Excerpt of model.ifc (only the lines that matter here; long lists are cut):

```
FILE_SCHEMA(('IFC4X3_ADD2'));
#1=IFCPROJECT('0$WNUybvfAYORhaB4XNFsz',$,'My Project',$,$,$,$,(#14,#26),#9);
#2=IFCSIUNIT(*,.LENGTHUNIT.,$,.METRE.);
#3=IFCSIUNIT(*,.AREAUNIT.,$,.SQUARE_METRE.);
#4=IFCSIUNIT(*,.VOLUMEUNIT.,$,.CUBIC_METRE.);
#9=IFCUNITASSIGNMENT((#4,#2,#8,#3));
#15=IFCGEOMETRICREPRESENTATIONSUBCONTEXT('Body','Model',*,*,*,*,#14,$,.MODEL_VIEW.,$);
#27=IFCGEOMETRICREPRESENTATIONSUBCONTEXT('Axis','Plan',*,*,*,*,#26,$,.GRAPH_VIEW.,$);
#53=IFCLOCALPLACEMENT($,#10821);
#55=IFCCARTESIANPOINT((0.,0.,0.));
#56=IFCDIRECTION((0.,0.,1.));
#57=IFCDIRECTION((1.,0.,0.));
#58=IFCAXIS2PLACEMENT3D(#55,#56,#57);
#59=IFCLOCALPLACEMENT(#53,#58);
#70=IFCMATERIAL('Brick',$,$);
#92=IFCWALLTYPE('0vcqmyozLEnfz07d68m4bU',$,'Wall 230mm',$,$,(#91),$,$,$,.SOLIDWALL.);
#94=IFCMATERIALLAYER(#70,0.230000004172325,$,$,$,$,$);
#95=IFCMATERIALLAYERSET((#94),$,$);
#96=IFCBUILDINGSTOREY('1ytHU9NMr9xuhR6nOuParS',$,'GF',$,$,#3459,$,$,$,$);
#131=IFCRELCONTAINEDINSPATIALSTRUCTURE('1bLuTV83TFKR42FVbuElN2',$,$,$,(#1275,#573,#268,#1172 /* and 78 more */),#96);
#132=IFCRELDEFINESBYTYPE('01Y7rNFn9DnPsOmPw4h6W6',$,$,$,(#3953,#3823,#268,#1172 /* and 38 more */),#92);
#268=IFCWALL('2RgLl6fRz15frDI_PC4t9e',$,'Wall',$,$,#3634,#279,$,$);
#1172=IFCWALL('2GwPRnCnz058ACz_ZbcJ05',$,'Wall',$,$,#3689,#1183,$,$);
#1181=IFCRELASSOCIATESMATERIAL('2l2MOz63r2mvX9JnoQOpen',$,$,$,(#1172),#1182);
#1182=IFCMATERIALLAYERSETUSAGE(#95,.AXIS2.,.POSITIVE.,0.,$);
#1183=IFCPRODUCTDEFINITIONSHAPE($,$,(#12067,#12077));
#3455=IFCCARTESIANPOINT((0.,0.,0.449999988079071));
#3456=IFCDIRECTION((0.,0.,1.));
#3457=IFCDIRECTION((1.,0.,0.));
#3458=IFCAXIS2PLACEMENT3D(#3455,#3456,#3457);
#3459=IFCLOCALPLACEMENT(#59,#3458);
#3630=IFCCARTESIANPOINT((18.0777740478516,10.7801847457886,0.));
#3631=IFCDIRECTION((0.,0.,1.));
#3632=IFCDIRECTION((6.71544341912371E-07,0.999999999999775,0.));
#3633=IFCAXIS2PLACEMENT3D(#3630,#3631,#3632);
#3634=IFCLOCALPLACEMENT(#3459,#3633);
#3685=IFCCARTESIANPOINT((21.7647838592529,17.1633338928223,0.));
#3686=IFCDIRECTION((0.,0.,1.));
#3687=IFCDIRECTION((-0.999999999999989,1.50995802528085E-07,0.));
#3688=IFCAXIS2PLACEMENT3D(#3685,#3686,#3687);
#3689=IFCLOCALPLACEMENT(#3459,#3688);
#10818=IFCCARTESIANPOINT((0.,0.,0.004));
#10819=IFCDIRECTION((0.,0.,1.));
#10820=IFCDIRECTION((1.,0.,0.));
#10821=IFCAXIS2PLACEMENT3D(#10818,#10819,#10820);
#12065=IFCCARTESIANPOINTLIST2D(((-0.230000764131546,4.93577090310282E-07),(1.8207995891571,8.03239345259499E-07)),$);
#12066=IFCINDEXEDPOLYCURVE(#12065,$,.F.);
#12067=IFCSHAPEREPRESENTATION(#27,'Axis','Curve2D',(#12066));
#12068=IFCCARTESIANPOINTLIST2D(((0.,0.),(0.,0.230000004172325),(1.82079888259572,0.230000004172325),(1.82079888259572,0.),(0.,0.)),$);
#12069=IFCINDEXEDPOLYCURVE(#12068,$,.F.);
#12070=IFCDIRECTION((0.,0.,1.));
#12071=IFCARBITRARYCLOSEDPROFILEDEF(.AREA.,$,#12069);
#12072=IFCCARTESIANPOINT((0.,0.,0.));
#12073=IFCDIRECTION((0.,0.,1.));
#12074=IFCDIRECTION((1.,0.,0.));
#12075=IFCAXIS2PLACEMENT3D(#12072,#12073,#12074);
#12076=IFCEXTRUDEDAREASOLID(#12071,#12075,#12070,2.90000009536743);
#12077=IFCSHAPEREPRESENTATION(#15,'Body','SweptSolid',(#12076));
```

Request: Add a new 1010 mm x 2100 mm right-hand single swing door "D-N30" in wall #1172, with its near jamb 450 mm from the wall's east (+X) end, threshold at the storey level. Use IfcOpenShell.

```python
import numpy as np
import ifcopenshell
import ifcopenshell.api.feature
import ifcopenshell.api.geometry
import ifcopenshell.api.root
import ifcopenshell.api.spatial
import ifcopenshell.geom
import ifcopenshell.util.element
import ifcopenshell.util.placement
import ifcopenshell.util.representation
import ifcopenshell.util.shape
import ifcopenshell.util.unit

model = ifcopenshell.open("model.ifc")
unit_scale = ifcopenshell.util.unit.calculate_unit_scale(model)
settings = ifcopenshell.geom.settings()


def volume(element):
    """Net volume in cubic metres, openings subtracted."""
    shape = ifcopenshell.geom.create_shape(settings, element)
    return ifcopenshell.util.shape.get_volume(shape.geometry)


wall = model.by_id(1172)
storey = ifcopenshell.util.element.get_container(wall, ifc_class="IfcBuildingStorey")
context = ifcopenshell.util.representation.get_context(model, "Model", "Body", "MODEL_VIEW")
before = volume(wall)

width, height, from_end, sill = 1.01, 2.1, 0.45, 0.0  # metres

# The wall runs along its own X axis, and the end named is its -X end.
wall_shape = ifcopenshell.geom.create_shape(settings, wall)
x, y, z = ifcopenshell.util.shape.get_vertices(wall_shape.geometry).T
start = x.min() + from_end
face, thickness = float(y.min()), float(y.max() - y.min())
wall_matrix = ifcopenshell.util.placement.get_local_placement(wall.ObjectPlacement)
level = ifcopenshell.util.placement.get_local_placement(storey.ObjectPlacement)[2, 3]


def in_wall(x, y):
    """Placement at x, y metres in the wall's axes, at sill height."""
    matrix = wall_matrix.copy()
    matrix[:, 3] = wall_matrix @ np.array([x / unit_scale, y / unit_scale, 0.0, 1.0])
    matrix[2, 3] = level + sill / unit_scale
    return matrix


# Opening: a box that overshoots both wall faces by 50 mm.
opening = ifcopenshell.api.root.create_entity(model, ifc_class="IfcOpeningElement", predefined_type="OPENING")
box = ifcopenshell.api.geometry.add_wall_representation(
    model, context=context, length=width, height=height, thickness=thickness + 0.1
)
ifcopenshell.api.geometry.assign_representation(model, product=opening, representation=box)
ifcopenshell.api.geometry.edit_object_placement(model, product=opening, matrix=in_wall(start, face - 0.05), is_si=False)
ifcopenshell.api.feature.add_feature(model, feature=opening, element=wall)

door = ifcopenshell.api.root.create_entity(model, ifc_class="IfcDoor", name="D-N30", predefined_type="DOOR")
door.OverallWidth, door.OverallHeight = width / unit_scale, height / unit_scale
door.OperationType = "SINGLE_SWING_RIGHT"
body = ifcopenshell.api.geometry.add_door_representation(
    model,
    context=context,
    overall_width=door.OverallWidth,
    overall_height=door.OverallHeight,
    operation_type="SINGLE_SWING_RIGHT",
    lining_properties={"LiningDepth": thickness / unit_scale, "ThresholdDepth": thickness / unit_scale},
)
ifcopenshell.api.geometry.assign_representation(model, product=door, representation=body)
ifcopenshell.api.spatial.assign_container(model, products=[door], relating_structure=storey)
ifcopenshell.api.feature.add_filling(model, opening=opening, element=door)

# The lining spans the wall, so the door starts at the wall face.
ifcopenshell.api.geometry.edit_object_placement(model, product=door, matrix=in_wall(start, face), is_si=False)

after = volume(wall)

print(f"wall volume {before:.3f} -> {after:.3f} m3")

model.write("model_v2.ifc")
```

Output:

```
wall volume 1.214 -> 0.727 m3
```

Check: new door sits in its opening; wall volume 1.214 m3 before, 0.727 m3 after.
